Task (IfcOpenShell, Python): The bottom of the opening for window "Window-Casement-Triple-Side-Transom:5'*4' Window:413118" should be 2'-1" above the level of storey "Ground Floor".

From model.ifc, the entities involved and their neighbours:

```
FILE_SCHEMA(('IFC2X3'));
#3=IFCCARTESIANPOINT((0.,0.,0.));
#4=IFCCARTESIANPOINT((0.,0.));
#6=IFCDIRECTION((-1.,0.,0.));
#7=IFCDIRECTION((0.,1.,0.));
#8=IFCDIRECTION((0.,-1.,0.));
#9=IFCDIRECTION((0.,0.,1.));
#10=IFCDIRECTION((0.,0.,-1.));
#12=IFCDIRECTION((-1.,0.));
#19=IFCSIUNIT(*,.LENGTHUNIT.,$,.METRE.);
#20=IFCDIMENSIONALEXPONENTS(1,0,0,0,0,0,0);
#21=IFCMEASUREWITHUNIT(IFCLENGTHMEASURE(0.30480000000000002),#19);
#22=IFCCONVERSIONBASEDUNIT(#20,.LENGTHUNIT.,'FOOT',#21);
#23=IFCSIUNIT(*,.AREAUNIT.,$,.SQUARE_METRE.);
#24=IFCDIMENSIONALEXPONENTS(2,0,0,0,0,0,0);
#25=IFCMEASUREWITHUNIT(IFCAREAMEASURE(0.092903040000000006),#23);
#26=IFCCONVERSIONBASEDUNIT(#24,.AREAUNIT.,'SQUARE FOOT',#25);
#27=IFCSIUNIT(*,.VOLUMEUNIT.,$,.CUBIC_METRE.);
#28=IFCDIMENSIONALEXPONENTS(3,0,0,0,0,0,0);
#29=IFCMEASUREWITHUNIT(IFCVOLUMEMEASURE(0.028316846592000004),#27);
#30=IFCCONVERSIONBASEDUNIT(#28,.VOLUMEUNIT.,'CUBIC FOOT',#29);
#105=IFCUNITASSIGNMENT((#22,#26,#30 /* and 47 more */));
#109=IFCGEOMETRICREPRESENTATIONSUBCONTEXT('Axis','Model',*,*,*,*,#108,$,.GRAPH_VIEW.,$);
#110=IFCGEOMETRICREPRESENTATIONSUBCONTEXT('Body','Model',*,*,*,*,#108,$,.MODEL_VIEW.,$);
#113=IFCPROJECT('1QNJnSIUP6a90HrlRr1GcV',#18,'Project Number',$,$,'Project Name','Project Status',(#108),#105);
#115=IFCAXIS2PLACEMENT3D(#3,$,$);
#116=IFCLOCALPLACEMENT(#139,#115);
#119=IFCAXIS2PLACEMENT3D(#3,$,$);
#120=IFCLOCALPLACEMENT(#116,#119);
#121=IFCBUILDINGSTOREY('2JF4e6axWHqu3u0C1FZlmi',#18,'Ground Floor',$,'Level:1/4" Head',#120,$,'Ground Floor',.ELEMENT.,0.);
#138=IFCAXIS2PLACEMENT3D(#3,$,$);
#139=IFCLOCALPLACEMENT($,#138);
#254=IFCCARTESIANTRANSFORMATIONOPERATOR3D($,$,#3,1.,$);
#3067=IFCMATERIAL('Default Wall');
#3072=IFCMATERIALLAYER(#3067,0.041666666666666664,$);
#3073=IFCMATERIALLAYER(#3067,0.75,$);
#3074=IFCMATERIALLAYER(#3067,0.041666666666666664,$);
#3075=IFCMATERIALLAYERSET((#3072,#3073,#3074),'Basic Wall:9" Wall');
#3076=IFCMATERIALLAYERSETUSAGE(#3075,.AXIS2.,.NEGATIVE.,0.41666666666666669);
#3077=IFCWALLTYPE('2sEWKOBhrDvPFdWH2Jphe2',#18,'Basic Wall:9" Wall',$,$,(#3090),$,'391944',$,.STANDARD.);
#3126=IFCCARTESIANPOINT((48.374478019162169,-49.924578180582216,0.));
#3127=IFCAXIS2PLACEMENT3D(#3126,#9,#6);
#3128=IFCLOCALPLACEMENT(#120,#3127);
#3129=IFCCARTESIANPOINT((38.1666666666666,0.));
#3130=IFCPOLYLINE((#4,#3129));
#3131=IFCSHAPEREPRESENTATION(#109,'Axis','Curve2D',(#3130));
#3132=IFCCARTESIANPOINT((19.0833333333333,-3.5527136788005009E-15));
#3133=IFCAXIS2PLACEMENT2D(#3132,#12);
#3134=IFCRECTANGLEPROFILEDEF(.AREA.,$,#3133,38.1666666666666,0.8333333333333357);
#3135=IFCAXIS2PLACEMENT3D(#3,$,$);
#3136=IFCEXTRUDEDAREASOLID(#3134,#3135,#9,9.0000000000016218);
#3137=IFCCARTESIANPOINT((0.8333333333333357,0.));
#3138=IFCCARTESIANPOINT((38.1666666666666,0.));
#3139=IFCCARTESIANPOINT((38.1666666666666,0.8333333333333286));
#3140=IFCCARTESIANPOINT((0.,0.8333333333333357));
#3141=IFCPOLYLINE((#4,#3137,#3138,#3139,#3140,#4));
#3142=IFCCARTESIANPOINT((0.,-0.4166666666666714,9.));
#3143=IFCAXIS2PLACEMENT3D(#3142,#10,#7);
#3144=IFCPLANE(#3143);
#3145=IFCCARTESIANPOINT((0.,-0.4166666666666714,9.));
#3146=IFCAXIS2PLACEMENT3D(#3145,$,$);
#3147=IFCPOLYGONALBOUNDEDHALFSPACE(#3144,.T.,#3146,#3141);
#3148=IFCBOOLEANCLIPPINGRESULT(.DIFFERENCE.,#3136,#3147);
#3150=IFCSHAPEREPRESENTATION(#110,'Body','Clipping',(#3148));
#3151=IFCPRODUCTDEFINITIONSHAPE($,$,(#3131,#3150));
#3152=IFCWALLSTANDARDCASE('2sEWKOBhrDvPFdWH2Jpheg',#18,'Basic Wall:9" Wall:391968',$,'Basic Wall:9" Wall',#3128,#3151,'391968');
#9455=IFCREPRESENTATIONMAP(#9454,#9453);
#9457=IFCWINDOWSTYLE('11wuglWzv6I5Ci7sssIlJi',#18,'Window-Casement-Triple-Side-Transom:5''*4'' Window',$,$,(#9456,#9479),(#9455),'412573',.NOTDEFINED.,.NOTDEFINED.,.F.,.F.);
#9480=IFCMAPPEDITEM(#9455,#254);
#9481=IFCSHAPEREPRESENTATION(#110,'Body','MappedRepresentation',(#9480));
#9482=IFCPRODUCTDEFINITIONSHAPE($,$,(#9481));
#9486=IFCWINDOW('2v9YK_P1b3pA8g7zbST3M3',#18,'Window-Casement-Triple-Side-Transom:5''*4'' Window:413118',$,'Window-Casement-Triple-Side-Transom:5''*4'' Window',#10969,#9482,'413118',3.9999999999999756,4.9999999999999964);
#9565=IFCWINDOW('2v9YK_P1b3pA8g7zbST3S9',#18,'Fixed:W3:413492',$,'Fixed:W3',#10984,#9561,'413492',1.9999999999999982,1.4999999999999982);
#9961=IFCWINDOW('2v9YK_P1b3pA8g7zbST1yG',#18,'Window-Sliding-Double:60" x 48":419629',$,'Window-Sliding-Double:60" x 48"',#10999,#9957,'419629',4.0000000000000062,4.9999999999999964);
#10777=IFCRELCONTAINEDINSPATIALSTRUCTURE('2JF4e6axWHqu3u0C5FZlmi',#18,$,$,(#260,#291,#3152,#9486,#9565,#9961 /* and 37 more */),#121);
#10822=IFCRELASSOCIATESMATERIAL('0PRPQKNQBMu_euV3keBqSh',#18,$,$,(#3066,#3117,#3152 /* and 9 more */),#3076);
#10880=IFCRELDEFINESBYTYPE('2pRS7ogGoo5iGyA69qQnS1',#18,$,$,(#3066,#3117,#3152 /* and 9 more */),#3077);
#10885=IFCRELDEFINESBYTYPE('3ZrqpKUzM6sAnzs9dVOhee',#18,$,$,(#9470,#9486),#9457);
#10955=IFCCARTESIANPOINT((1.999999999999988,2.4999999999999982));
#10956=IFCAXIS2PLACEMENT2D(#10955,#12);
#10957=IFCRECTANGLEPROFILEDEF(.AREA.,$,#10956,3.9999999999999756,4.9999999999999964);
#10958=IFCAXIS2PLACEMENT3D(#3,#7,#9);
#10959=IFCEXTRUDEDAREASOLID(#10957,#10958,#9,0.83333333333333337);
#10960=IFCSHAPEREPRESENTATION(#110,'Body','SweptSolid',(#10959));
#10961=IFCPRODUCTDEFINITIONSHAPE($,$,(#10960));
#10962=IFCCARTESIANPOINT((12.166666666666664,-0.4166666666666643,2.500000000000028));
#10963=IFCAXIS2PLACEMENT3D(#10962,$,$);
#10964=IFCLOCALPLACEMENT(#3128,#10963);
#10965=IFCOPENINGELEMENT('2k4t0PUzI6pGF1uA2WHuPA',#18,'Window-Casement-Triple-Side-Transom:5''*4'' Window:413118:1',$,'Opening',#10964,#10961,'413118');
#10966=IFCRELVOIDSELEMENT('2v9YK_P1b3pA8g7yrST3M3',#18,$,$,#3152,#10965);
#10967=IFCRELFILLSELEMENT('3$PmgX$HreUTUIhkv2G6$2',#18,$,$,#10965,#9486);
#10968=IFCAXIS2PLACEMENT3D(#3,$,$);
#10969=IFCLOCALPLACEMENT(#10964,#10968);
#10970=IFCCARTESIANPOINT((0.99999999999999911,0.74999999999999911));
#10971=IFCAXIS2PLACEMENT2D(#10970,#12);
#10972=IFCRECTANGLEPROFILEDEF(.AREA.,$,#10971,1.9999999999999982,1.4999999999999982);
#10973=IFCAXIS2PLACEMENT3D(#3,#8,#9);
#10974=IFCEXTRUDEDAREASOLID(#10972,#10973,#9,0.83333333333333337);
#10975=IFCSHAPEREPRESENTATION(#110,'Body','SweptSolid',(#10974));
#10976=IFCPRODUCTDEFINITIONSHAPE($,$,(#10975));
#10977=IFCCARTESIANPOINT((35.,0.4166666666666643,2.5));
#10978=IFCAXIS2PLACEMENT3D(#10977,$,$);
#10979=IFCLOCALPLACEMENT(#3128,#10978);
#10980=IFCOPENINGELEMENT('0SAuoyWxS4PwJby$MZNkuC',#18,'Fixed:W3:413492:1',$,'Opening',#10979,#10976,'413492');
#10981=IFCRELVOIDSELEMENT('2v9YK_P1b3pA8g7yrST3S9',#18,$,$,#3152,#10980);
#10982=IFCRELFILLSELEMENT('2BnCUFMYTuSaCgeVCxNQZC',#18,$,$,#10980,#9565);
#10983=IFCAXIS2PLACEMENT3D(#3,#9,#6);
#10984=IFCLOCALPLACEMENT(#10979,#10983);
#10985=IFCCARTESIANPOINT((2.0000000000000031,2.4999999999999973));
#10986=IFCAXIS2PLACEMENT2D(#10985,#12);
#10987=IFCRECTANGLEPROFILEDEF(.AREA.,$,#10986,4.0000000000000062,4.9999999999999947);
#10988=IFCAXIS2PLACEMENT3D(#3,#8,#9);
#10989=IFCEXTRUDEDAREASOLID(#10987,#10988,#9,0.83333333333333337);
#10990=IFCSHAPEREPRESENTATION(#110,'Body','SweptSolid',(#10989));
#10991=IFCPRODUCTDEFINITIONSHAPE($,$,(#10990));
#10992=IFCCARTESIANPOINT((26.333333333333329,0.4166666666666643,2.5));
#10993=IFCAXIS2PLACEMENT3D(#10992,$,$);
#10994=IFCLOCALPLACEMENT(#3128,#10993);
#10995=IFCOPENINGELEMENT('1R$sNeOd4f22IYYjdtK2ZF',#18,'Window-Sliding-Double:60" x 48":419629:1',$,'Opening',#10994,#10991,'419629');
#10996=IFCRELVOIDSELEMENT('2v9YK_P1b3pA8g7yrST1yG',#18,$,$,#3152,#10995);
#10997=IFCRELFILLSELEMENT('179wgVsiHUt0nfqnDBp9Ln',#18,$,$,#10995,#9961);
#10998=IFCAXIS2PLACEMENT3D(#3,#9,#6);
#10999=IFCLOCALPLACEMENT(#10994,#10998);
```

```python
import numpy as np
import ifcopenshell
import ifcopenshell.api.geometry
import ifcopenshell.geom
import ifcopenshell.util.element
import ifcopenshell.util.placement
import ifcopenshell.util.shape
import ifcopenshell.util.unit

model = ifcopenshell.open("model.ifc")
unit_scale = ifcopenshell.util.unit.calculate_unit_scale(model)

window = model.by_guid("2v9YK_P1b3pA8g7zbST3M3")
opening = window.FillsVoids[0].RelatingOpeningElement
storey = ifcopenshell.util.element.get_container(window, ifc_class="IfcBuildingStorey")
level = ifcopenshell.util.placement.get_local_placement(storey.ObjectPlacement)[2, 3]

# The opening's origin need not be at the sill, so measure its lowest point.
shape = ifcopenshell.geom.create_shape(ifcopenshell.geom.settings(), opening)
bottom = ifcopenshell.util.shape.get_shape_bottom_elevation(shape, shape.geometry) / unit_scale
dz = level + 25 * 0.0254 / unit_scale - bottom

shift = np.array([0.0, 0.0, dz])
# The window is placed relative to its opening, so it follows when the opening moves.
matrix = ifcopenshell.util.placement.get_local_placement(opening.ObjectPlacement)
matrix[:3, 3] += shift
ifcopenshell.api.geometry.edit_object_placement(
    model, product=opening, matrix=matrix, is_si=False, should_transform_children=True
)

print(f"moved by {dz * unit_scale:+.3f} m")

model.write("model_v2.ifc")
```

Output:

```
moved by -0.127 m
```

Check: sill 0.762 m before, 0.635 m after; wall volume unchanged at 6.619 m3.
